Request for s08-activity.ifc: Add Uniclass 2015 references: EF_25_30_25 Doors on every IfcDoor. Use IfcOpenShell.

First a look at what the model holds.

```python
import ifcopenshell

model = ifcopenshell.open("s08-activity.ifc")
print(model.schema)
print("classifications:", [c.Name for c in model.by_type("IfcClassification")])
for ifc_class in ("IfcDoor", "IfcRoof", "IfcStair", "IfcWall", "IfcWindow"):
    print(ifc_class, len(model.by_type(ifc_class)))
```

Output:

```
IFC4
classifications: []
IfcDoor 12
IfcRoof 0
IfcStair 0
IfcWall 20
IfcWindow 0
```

```python
import ifcopenshell
import ifcopenshell.api.classification

model = ifcopenshell.open("s08-activity.ifc")

system = ifcopenshell.api.classification.add_classification(model, classification="Uniclass 2015")

codes = {
    "IfcDoor": ("EF_25_30_25", "Doors"),
}
for ifc_class, (code, name) in codes.items():
    products = model.by_type(ifc_class)
    ifcopenshell.api.classification.add_reference(
        model, products=products, classification=system, identification=code, name=name
    )
    print(code, len(products))

model.write("s08-activity-out.ifc")
```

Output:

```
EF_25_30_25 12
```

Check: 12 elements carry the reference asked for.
